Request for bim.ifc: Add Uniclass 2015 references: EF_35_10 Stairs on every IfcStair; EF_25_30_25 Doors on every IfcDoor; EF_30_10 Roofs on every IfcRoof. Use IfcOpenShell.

First a look at what the model holds.

```python
import ifcopenshell

model = ifcopenshell.open("bim.ifc")
print(model.schema)
print("classifications:", [c.Name for c in model.by_type("IfcClassification")])
for ifc_class in ("IfcDoor", "IfcRoof", "IfcStair", "IfcWall", "IfcWindow"):
    print(ifc_class, len(model.by_type(ifc_class)))
```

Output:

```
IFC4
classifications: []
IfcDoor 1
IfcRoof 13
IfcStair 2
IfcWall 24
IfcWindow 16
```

```python
import ifcopenshell
import ifcopenshell.api.classification

model = ifcopenshell.open("bim.ifc")

system = ifcopenshell.api.classification.add_classification(model, classification="Uniclass 2015")

codes = {
    "IfcStair": ("EF_35_10", "Stairs"),
    "IfcDoor": ("EF_25_30_25", "Doors"),
    "IfcRoof": ("EF_30_10", "Roofs"),
}
for ifc_class, (code, name) in codes.items():
    products = model.by_type(ifc_class)
    ifcopenshell.api.classification.add_reference(
        model, products=products, classification=system, identification=code, name=name
    )
    print(code, len(products))

model.write("bim_updated.ifc")
```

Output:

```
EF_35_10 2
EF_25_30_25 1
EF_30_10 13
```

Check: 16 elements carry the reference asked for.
